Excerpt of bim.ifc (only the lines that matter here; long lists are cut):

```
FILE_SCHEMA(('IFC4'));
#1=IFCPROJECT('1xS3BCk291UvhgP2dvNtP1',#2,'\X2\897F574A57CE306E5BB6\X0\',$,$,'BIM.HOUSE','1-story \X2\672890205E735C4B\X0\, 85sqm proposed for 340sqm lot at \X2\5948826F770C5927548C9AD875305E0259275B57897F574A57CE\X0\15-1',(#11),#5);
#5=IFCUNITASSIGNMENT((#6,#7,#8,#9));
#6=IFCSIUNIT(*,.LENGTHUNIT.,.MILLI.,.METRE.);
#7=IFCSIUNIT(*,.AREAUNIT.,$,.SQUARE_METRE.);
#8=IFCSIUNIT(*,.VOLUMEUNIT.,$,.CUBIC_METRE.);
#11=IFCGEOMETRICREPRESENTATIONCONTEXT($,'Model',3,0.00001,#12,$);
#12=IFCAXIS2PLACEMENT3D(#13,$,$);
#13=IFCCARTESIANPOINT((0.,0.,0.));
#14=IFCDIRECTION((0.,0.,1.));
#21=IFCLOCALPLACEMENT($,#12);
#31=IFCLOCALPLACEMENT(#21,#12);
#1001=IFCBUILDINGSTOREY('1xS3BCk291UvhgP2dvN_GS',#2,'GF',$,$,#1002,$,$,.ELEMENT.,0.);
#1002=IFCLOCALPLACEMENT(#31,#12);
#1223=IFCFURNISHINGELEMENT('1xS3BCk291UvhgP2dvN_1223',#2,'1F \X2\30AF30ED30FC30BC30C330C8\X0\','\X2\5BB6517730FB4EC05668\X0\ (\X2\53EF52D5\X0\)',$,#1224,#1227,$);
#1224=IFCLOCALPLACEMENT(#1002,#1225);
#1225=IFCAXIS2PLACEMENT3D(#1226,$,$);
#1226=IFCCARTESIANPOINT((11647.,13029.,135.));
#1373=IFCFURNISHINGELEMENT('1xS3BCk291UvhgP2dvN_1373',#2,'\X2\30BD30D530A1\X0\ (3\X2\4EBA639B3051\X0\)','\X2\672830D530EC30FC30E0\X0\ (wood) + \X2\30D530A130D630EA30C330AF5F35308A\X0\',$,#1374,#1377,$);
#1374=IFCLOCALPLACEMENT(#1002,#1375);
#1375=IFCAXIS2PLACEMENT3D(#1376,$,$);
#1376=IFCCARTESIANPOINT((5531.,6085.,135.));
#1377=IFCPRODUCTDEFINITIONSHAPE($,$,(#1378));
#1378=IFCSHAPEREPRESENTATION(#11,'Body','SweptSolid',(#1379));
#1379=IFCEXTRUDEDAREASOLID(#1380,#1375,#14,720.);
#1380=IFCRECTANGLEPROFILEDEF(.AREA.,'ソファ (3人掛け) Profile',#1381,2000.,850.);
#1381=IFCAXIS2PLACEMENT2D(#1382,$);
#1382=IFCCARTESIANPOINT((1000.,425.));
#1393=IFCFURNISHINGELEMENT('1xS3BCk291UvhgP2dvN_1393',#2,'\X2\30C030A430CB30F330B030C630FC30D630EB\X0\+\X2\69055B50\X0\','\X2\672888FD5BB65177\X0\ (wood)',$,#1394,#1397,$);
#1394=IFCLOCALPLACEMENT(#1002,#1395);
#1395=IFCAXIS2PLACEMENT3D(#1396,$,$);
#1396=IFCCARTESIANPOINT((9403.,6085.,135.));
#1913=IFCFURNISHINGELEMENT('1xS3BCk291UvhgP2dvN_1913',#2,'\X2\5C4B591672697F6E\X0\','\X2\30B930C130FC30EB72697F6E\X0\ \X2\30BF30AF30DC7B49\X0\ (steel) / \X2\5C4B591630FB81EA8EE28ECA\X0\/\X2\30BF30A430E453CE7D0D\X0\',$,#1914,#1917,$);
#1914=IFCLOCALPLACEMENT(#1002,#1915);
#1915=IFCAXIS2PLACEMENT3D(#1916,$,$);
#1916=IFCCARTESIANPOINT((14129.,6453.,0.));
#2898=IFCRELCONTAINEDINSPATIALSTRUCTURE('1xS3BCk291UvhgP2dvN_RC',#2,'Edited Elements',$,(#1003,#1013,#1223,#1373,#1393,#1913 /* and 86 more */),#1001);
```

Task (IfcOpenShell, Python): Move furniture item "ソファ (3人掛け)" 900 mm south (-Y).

```python
import ifcopenshell
import ifcopenshell.api.geometry
import ifcopenshell.util.placement

model = ifcopenshell.open("bim.ifc")

item = model.by_id(1373)
matrix = ifcopenshell.util.placement.get_local_placement(item.ObjectPlacement)
matrix[1, 3] -= 900.0
ifcopenshell.api.geometry.edit_object_placement(model, product=item, matrix=matrix, is_si=False)

print(ifcopenshell.util.placement.get_local_placement(item.ObjectPlacement).round(3) + 0.0)

model.write("bim_rev.ifc")
```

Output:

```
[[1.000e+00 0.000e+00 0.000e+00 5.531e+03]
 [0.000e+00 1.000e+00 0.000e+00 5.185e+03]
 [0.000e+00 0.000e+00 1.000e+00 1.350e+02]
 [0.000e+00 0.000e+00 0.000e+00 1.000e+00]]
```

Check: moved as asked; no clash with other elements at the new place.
